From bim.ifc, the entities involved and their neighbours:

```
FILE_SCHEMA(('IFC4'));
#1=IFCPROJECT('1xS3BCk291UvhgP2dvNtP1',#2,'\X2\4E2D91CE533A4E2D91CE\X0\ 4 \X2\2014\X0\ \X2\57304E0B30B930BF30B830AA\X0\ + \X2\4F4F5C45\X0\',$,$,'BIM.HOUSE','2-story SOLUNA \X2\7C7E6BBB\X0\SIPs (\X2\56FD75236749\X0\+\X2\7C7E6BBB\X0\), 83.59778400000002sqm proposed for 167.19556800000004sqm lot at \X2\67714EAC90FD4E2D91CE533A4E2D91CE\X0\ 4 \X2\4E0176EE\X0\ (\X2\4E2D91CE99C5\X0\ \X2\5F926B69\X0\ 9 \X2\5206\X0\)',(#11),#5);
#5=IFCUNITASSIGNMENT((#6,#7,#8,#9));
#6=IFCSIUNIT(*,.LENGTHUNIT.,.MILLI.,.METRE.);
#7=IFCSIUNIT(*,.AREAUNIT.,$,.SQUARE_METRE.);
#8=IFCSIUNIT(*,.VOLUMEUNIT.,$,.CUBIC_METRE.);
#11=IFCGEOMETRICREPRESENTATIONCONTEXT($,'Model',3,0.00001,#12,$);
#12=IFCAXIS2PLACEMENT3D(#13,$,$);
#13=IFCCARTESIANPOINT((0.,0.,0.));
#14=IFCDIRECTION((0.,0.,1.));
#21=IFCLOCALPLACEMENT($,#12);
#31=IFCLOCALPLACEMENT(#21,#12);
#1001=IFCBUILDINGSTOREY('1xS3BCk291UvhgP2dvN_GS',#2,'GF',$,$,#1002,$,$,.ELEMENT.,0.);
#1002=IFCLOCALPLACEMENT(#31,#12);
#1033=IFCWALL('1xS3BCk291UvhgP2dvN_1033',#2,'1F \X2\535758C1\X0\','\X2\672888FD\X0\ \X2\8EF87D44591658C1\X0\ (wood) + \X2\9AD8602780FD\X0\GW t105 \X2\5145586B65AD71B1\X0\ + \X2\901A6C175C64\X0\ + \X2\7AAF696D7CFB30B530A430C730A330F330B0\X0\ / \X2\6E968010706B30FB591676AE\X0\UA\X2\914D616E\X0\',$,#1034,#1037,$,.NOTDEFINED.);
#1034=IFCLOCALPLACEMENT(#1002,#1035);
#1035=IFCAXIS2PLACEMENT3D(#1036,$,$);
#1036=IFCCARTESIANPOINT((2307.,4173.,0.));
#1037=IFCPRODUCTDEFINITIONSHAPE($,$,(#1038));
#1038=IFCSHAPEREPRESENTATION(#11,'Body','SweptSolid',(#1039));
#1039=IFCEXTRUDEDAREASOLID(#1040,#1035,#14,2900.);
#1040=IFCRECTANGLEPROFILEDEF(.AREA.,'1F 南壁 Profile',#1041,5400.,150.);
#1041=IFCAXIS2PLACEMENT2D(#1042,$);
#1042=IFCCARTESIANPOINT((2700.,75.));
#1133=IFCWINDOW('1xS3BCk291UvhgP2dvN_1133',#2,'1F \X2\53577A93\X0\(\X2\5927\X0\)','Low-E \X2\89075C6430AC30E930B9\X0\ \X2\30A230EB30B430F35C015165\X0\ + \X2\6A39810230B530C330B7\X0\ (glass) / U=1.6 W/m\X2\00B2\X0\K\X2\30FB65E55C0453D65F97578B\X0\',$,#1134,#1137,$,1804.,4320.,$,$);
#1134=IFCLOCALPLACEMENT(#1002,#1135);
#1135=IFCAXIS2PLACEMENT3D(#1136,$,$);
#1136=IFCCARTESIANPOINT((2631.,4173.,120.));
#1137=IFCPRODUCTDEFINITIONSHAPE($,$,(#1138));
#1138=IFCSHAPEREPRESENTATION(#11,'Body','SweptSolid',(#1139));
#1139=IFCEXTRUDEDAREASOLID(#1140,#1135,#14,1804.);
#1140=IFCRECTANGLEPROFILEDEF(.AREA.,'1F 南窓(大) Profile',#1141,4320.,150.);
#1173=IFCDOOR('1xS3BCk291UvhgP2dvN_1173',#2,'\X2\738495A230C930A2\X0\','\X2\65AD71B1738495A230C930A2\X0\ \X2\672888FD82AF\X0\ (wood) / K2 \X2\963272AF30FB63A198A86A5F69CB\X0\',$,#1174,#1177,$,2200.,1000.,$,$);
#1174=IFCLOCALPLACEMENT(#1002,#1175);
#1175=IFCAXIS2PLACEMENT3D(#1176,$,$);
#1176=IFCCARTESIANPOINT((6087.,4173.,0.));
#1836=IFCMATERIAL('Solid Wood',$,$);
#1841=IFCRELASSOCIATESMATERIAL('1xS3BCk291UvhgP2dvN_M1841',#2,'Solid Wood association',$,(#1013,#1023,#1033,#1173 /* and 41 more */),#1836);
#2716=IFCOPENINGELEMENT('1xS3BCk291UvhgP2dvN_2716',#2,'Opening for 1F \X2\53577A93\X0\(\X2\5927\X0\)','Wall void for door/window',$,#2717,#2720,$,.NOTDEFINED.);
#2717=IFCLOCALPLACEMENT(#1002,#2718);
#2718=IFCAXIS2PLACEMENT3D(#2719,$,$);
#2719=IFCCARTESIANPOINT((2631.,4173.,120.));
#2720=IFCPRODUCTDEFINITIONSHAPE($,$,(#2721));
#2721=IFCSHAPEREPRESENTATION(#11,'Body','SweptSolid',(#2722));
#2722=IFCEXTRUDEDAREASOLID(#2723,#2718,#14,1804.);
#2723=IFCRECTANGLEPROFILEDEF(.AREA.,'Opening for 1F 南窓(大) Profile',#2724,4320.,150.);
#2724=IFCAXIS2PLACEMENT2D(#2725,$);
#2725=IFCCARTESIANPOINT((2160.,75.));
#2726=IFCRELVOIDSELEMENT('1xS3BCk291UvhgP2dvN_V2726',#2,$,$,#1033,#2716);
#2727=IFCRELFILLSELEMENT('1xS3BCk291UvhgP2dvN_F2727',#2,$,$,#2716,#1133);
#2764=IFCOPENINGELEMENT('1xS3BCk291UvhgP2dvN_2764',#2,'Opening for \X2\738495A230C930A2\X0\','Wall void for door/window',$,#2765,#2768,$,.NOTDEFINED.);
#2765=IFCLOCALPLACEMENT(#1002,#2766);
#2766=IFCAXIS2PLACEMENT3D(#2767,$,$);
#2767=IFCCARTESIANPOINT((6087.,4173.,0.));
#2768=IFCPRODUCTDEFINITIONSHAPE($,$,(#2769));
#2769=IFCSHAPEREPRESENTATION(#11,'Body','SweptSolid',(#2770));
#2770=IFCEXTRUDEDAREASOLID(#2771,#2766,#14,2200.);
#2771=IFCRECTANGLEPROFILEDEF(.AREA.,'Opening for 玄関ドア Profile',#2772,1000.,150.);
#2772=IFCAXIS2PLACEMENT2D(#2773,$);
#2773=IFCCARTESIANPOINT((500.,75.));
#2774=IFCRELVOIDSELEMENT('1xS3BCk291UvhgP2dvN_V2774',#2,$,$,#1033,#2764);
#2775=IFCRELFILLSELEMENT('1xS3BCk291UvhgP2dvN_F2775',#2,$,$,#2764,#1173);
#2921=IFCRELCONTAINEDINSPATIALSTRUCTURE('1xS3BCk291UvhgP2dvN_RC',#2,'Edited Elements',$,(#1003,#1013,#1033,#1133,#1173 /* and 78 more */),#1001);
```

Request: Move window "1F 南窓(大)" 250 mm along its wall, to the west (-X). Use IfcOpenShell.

```python
import ifcopenshell
import ifcopenshell.api.geometry
import ifcopenshell.util.placement
import ifcopenshell.util.unit

model = ifcopenshell.open("bim.ifc")
unit_scale = ifcopenshell.util.unit.calculate_unit_scale(model)

window = model.by_id(1133)
opening = window.FillsVoids[0].RelatingOpeningElement
wall = opening.VoidsElements[0].RelatingBuildingElement

wall_matrix = ifcopenshell.util.placement.get_local_placement(wall.ObjectPlacement)
shift = wall_matrix[:3, 0] * -0.25 / unit_scale
before = ifcopenshell.util.placement.get_local_placement(window.ObjectPlacement)[:3, 3].copy()

# The window is not placed relative to its opening, so move both.
for product in (opening, window):
    matrix = ifcopenshell.util.placement.get_local_placement(product.ObjectPlacement)
    matrix[:3, 3] += shift
    ifcopenshell.api.geometry.edit_object_placement(model, product=product, matrix=matrix, is_si=False)

after = ifcopenshell.util.placement.get_local_placement(window.ObjectPlacement)[:3, 3]
print("window moved by", (after - before).round(3) + 0.0)

model.write("bim_rev.ifc")
```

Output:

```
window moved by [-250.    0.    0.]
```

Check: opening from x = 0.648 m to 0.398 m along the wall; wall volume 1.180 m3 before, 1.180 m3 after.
